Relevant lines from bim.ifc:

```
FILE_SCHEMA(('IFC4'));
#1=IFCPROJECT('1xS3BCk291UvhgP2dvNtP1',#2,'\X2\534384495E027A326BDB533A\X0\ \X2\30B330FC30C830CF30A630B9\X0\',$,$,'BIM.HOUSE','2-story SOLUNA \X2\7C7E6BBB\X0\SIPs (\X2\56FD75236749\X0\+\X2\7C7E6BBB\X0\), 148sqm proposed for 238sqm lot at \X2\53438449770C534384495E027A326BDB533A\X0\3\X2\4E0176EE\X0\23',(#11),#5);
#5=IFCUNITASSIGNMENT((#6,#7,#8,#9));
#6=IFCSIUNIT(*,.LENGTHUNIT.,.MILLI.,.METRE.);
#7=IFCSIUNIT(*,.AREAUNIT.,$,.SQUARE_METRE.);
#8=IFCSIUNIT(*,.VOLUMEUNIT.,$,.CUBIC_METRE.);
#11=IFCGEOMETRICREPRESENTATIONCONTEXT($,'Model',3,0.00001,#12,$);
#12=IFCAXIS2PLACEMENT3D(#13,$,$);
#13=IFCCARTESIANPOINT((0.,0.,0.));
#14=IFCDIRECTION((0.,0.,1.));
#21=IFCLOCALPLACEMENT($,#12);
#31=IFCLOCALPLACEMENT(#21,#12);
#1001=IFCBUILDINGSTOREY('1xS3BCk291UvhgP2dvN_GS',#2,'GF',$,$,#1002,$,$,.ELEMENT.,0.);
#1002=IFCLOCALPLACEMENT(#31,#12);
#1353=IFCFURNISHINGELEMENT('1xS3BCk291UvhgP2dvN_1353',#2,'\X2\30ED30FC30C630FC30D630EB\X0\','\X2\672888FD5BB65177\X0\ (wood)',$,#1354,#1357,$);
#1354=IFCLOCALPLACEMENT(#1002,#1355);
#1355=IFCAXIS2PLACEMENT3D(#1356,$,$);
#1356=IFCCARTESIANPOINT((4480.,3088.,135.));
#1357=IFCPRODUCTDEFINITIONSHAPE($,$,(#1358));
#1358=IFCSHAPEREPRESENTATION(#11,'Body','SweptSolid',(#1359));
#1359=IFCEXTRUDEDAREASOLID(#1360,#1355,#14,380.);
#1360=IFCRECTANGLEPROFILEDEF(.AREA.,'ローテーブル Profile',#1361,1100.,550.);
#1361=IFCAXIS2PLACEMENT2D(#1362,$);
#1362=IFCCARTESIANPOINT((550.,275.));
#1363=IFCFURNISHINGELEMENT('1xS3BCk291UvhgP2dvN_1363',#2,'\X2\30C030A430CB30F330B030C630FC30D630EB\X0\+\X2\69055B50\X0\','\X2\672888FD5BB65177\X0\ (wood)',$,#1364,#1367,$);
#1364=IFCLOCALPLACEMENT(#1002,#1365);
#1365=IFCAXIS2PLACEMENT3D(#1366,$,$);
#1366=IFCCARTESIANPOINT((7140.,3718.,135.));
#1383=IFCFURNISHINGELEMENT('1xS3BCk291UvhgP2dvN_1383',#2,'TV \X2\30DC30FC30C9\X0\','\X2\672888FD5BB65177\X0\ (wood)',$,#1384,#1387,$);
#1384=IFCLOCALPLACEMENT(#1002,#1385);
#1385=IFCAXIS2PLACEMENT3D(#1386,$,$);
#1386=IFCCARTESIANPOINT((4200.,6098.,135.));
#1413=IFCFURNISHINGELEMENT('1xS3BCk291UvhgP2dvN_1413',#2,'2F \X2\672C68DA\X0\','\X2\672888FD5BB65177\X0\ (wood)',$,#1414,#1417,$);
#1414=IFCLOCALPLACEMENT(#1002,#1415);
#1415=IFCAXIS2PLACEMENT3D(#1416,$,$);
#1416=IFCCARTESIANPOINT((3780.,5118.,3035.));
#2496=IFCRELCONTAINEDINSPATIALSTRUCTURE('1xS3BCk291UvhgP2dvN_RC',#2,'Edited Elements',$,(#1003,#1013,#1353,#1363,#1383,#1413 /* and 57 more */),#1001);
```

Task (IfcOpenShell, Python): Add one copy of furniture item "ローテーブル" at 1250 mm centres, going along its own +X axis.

```python
import ifcopenshell
import ifcopenshell.api.geometry
import ifcopenshell.api.root
import ifcopenshell.util.element
import ifcopenshell.util.placement

model = ifcopenshell.open("bim.ifc")


def reuse_history(source, copy):
    """copy_class also copies each property set's owner history, people and application; keep the originals."""
    for rel in copy.IsDefinedBy:
        if rel.is_a("IfcRelDefinesByProperties") and (history := rel.RelatingPropertyDefinition.OwnerHistory):
            rel.RelatingPropertyDefinition.OwnerHistory = source.OwnerHistory
            ifcopenshell.util.element.remove_deep2(model, history)


source = model.by_guid("1xS3BCk291UvhgP2dvN_1353")
base = ifcopenshell.util.placement.get_local_placement(source.ObjectPlacement)
step = base[:3, 0] * 1250.0

for i in range(1, 2):
    copy = ifcopenshell.api.root.copy_class(model, product=source)
    copy.Representation = ifcopenshell.util.element.copy_deep(
        model, source.Representation, exclude=["IfcGeometricRepresentationContext", "IfcRepresentationMap"]
    )
    reuse_history(source, copy)
    matrix = base.copy()
    matrix[:3, 3] += i * step
    print("added at", matrix[:3, 3].round(3) + 0.0)
    ifcopenshell.api.geometry.edit_object_placement(model, product=copy, matrix=matrix, is_si=False)

model.write("bim_updated.ifc")
```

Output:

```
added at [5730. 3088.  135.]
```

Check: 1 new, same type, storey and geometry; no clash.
